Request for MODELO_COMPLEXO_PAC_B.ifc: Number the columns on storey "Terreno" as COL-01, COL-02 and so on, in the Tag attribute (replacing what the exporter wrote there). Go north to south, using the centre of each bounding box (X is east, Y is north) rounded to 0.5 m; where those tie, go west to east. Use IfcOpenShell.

First a look at what the model holds.

```python
import ifcopenshell
import ifcopenshell.util.element
import ifcopenshell.util.placement

model = ifcopenshell.open("MODELO_COMPLEXO_PAC_B.ifc")
print(model.schema)
storey = next(s for s in model.by_type("IfcBuildingStorey") if s.Name == "Terreno")
columns = [e for e in ifcopenshell.util.element.get_decomposition(storey) if e.is_a("IfcColumn")]
for e in sorted(columns, key=lambda e: e.id()):
    origin = ifcopenshell.util.placement.get_local_placement(e.ObjectPlacement)[:3, 3]
    print(e.id(), e.Tag, e.Name, origin.round(2) + 0.0, sep=" | ")
```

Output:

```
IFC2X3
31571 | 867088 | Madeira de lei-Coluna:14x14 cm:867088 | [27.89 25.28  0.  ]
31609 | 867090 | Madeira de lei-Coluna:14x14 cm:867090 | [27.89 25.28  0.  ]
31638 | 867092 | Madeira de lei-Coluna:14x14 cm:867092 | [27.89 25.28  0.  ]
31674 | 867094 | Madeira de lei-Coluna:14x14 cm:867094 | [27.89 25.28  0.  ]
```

```python
import ifcopenshell
import ifcopenshell.geom
import ifcopenshell.util.element
import ifcopenshell.util.shape

model = ifcopenshell.open("MODELO_COMPLEXO_PAC_B.ifc")
settings = ifcopenshell.geom.settings()
settings.set("use-world-coords", True)


def centre(element):
    shape = ifcopenshell.geom.create_shape(settings, element)
    return ifcopenshell.util.shape.get_bbox_centroid(shape.geometry)


storey = next(s for s in model.by_type("IfcBuildingStorey") if s.Name == "Terreno")
columns = [e for e in ifcopenshell.util.element.get_decomposition(storey) if e.is_a("IfcColumn")]

# Insertion points can sit at a corner or the storey origin, so sort by the geometry (in metres).
centres = {e: centre(e) for e in columns}
columns.sort(key=lambda e: (-round(centres[e][1] / 0.5), centres[e][0]))

for i, e in enumerate(columns, start=1):
    number = f"COL-{i:02d}"
    e.Tag = number
    print(e.id(), number)

model.write("MODELO_COMPLEXO_PAC_B_v2.ifc")
```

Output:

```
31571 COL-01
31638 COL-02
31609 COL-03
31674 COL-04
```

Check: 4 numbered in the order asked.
